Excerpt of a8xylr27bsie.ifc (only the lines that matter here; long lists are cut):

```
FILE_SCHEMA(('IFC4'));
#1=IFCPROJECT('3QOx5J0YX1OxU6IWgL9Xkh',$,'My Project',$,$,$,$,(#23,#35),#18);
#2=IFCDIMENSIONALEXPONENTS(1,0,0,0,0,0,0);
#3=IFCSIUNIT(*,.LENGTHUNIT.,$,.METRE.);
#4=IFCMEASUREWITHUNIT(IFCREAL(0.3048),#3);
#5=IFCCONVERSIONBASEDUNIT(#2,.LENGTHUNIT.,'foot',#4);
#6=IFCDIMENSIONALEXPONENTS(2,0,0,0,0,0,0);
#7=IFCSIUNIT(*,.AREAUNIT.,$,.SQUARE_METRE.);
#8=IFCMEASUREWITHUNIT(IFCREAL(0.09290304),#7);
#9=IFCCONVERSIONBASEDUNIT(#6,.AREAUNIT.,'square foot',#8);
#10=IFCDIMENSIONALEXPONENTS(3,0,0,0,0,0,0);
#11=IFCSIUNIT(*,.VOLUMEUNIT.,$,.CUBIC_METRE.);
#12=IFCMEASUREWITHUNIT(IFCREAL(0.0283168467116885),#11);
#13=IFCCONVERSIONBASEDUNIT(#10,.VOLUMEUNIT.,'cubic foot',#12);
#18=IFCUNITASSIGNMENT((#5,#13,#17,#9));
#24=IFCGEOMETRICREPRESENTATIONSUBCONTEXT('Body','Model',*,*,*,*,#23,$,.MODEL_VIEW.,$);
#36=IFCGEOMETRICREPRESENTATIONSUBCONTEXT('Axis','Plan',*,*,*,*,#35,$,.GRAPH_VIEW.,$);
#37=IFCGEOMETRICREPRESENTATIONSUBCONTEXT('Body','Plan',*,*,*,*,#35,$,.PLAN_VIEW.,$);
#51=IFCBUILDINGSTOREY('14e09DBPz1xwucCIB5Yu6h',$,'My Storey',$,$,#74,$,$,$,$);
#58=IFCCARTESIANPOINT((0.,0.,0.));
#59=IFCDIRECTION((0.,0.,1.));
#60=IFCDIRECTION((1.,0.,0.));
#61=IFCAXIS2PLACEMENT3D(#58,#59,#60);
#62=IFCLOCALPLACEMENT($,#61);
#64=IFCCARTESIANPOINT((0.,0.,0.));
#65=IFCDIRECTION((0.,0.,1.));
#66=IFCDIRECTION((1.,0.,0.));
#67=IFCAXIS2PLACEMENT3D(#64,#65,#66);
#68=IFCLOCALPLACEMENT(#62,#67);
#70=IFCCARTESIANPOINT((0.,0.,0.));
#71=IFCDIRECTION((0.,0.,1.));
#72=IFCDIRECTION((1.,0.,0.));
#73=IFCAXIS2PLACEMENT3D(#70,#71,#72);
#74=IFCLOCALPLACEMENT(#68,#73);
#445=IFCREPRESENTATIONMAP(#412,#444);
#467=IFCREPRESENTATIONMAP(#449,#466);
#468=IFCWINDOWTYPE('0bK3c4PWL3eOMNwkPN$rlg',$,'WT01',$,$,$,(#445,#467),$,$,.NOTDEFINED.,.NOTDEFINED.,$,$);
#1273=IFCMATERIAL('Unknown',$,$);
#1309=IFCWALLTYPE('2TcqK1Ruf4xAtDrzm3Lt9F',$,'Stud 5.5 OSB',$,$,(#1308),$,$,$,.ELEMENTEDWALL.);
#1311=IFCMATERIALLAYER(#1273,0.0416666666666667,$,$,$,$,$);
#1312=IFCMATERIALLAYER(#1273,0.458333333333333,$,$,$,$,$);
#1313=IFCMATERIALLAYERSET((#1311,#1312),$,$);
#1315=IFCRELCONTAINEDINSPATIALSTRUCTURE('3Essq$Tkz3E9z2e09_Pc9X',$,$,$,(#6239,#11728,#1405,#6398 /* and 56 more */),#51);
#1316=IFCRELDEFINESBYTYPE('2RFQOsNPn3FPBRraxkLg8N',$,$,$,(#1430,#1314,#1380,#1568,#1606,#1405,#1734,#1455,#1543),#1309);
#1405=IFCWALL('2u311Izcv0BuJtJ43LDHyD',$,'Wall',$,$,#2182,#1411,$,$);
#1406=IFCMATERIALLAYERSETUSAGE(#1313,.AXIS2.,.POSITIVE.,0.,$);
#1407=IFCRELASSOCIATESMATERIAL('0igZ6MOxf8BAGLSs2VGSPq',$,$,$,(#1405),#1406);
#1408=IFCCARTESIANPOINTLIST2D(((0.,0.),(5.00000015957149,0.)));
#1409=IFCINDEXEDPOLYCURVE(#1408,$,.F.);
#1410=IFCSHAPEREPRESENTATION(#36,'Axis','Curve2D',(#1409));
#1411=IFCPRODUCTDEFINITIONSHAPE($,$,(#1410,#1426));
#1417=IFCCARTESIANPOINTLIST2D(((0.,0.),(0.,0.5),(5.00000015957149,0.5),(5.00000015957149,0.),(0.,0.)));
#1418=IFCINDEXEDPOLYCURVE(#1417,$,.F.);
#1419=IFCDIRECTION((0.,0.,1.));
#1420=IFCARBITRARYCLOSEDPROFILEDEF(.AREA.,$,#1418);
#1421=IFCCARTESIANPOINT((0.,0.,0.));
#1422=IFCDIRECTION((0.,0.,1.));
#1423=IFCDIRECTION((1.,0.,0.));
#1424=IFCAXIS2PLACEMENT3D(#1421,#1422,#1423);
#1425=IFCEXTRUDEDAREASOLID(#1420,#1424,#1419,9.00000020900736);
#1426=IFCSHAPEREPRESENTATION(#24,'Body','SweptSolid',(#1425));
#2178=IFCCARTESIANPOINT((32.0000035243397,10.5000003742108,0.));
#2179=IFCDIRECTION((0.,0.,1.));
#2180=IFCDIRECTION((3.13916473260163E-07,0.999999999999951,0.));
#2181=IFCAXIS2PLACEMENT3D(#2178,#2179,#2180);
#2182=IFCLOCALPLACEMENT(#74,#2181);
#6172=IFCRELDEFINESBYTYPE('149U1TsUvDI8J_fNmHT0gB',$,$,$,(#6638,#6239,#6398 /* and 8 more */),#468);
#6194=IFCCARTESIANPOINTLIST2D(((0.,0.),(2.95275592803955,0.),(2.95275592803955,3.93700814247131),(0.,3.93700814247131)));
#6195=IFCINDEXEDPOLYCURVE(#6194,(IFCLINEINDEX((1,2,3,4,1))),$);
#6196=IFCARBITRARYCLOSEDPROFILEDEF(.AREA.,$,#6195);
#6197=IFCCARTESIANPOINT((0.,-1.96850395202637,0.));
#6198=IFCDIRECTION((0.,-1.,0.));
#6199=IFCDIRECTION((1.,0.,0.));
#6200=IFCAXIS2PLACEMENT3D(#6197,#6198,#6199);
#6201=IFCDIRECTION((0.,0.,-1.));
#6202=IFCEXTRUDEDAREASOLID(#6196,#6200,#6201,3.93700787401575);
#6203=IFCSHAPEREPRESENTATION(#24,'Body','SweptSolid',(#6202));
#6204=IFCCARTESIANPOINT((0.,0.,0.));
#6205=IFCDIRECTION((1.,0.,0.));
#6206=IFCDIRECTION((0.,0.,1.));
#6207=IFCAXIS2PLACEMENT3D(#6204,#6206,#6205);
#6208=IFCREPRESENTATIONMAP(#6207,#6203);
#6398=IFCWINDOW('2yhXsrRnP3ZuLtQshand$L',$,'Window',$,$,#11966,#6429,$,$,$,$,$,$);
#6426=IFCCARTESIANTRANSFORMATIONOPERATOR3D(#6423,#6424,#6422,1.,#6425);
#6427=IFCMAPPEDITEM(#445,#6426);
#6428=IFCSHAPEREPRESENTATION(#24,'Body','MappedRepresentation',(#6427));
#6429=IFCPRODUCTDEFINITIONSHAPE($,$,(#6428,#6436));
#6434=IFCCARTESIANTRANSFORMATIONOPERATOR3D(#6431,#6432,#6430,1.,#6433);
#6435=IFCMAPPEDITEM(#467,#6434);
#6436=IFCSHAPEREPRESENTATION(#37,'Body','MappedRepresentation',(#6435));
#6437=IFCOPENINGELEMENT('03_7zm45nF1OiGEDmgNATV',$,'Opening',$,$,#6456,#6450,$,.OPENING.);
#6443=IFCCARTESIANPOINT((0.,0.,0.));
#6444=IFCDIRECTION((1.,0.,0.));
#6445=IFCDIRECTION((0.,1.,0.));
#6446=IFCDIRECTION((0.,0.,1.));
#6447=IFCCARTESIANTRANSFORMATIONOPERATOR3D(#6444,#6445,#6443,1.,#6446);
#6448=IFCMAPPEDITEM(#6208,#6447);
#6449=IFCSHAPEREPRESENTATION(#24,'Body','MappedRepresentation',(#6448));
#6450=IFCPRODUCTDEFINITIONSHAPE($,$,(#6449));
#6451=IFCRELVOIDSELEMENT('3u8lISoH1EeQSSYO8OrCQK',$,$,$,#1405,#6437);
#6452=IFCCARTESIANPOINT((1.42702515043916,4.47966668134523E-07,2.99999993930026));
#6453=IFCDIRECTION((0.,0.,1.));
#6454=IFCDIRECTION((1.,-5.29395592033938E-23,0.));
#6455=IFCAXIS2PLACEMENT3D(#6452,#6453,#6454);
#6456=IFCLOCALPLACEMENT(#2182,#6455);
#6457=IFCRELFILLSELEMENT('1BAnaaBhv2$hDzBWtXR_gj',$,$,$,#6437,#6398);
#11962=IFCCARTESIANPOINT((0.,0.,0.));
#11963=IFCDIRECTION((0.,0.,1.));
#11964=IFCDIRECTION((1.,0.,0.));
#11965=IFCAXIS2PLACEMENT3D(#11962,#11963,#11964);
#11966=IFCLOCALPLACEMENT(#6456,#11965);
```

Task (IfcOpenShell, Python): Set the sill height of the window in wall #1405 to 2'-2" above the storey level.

```python
import numpy as np
import ifcopenshell
import ifcopenshell.api.geometry
import ifcopenshell.geom
import ifcopenshell.util.element
import ifcopenshell.util.placement
import ifcopenshell.util.shape
import ifcopenshell.util.unit

model = ifcopenshell.open("a8xylr27bsie.ifc")
unit_scale = ifcopenshell.util.unit.calculate_unit_scale(model)

window = model.by_guid("2yhXsrRnP3ZuLtQshand$L")
opening = window.FillsVoids[0].RelatingOpeningElement
storey = ifcopenshell.util.element.get_container(window, ifc_class="IfcBuildingStorey")
level = ifcopenshell.util.placement.get_local_placement(storey.ObjectPlacement)[2, 3]

# The opening's origin need not be at the sill, so measure its lowest point.
shape = ifcopenshell.geom.create_shape(ifcopenshell.geom.settings(), opening)
bottom = ifcopenshell.util.shape.get_shape_bottom_elevation(shape, shape.geometry) / unit_scale
dz = level + 26 * 0.0254 / unit_scale - bottom

shift = np.array([0.0, 0.0, dz])
# The window is placed relative to its opening, so it follows when the opening moves.
matrix = ifcopenshell.util.placement.get_local_placement(opening.ObjectPlacement)
matrix[:3, 3] += shift
ifcopenshell.api.geometry.edit_object_placement(
    model, product=opening, matrix=matrix, is_si=False, should_transform_children=True
)

print(f"moved by {dz * unit_scale:+.3f} m")

model.write("a8xylr27bsie_rev.ifc")
```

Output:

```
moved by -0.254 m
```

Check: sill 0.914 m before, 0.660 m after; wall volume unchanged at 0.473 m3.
